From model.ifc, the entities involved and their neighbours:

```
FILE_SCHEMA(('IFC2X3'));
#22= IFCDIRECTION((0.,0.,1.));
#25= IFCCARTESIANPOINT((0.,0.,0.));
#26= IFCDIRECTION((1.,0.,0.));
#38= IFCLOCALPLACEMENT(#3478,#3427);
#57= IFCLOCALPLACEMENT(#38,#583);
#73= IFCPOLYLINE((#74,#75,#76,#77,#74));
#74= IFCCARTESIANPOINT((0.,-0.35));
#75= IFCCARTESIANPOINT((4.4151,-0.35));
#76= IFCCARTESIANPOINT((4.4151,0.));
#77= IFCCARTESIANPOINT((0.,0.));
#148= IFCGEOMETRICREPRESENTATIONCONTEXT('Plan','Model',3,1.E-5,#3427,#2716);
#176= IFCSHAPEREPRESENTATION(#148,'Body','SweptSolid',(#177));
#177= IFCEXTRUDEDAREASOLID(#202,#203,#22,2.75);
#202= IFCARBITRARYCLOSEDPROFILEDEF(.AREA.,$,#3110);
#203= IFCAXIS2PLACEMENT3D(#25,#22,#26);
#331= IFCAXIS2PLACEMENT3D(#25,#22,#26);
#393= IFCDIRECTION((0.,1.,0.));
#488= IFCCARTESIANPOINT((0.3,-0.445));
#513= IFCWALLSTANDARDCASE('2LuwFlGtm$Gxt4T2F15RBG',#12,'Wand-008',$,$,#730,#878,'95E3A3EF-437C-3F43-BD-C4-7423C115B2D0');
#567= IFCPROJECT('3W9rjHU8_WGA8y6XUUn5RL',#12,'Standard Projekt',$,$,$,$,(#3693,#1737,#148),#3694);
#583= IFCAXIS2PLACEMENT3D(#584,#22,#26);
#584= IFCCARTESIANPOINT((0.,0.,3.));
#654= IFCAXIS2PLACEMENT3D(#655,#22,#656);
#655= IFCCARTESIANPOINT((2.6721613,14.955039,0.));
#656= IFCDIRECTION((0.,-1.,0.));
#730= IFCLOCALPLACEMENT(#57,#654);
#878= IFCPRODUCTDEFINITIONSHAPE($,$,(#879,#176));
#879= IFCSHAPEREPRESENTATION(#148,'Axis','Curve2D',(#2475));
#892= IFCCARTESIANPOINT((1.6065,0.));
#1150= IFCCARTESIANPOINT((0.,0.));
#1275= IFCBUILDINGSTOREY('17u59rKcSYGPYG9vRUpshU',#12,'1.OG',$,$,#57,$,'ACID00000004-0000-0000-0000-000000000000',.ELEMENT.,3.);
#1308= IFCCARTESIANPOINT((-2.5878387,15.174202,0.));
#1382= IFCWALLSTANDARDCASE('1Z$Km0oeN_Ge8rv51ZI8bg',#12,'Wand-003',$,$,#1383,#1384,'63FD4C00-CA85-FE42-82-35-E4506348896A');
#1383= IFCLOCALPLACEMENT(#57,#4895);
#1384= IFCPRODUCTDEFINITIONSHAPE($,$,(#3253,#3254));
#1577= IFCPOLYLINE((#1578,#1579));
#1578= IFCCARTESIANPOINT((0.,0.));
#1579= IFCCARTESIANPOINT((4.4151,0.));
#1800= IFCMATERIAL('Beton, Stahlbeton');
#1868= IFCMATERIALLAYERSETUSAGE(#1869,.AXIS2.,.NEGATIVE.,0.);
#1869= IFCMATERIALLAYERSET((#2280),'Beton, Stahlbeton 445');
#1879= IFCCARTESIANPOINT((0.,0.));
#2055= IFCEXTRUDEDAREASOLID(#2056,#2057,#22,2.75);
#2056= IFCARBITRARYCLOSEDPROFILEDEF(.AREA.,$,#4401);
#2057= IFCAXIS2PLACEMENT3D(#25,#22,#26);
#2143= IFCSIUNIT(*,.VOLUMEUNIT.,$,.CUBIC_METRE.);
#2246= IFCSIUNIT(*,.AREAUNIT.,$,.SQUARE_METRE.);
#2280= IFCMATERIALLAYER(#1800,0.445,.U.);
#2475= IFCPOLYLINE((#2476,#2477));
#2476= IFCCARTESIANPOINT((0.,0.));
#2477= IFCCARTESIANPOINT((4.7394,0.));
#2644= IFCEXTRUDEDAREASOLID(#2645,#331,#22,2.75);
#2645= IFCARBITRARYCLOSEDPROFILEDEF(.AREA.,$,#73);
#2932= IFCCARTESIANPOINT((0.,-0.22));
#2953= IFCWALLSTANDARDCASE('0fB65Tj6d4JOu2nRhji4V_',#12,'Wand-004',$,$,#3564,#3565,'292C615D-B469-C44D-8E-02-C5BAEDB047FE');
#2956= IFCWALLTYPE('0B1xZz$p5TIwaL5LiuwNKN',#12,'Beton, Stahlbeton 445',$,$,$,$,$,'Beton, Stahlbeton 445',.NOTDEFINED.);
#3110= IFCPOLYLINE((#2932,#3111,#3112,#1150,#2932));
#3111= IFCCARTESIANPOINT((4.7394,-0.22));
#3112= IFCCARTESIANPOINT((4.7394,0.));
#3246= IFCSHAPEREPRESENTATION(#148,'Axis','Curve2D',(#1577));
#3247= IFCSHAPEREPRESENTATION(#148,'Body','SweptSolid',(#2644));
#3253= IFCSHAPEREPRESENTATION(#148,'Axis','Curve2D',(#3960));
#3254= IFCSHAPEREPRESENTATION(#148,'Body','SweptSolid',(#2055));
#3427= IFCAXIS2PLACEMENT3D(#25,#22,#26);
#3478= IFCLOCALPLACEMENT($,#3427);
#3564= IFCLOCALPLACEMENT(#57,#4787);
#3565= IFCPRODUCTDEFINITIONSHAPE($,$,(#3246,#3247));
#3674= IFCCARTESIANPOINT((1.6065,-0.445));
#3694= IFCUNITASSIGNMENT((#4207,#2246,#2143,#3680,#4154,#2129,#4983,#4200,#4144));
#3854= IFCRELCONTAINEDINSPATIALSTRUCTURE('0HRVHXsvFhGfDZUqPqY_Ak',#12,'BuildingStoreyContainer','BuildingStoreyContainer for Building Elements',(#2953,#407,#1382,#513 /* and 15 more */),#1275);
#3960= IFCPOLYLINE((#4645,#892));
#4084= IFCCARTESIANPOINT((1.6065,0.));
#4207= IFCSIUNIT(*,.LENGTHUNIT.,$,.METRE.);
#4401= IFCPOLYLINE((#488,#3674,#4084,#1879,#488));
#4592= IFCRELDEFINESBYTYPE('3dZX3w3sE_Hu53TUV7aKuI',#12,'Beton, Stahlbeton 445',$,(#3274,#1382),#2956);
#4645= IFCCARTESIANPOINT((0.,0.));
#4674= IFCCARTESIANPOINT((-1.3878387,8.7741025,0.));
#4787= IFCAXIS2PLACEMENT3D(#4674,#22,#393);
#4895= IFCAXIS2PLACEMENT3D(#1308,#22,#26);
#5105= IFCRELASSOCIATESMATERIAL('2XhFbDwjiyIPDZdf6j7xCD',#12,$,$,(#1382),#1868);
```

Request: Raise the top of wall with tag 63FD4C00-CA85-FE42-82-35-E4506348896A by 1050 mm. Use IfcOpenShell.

```python
import ifcopenshell
import ifcopenshell.geom
import ifcopenshell.util.shape

model = ifcopenshell.open("model.ifc")
settings = ifcopenshell.geom.settings()


def volume(element):
    """Net volume in cubic metres, openings subtracted."""
    shape = ifcopenshell.geom.create_shape(settings, element)
    return ifcopenshell.util.shape.get_volume(shape.geometry)


wall = model.by_id(1382)
before = volume(wall)

body = next(r for r in wall.Representation.Representations if r.RepresentationIdentifier == "Body")
solid = body.Items[0]
old_height = solid.Depth
solid.Depth += 1.05
after = volume(wall)

print(f"height {old_height:g} -> {solid.Depth:g}, volume {before:.3f} -> {after:.3f} m3")

model.write("model_v2.ifc")
```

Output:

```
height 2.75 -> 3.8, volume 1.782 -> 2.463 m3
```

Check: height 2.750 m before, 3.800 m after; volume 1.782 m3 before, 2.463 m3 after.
